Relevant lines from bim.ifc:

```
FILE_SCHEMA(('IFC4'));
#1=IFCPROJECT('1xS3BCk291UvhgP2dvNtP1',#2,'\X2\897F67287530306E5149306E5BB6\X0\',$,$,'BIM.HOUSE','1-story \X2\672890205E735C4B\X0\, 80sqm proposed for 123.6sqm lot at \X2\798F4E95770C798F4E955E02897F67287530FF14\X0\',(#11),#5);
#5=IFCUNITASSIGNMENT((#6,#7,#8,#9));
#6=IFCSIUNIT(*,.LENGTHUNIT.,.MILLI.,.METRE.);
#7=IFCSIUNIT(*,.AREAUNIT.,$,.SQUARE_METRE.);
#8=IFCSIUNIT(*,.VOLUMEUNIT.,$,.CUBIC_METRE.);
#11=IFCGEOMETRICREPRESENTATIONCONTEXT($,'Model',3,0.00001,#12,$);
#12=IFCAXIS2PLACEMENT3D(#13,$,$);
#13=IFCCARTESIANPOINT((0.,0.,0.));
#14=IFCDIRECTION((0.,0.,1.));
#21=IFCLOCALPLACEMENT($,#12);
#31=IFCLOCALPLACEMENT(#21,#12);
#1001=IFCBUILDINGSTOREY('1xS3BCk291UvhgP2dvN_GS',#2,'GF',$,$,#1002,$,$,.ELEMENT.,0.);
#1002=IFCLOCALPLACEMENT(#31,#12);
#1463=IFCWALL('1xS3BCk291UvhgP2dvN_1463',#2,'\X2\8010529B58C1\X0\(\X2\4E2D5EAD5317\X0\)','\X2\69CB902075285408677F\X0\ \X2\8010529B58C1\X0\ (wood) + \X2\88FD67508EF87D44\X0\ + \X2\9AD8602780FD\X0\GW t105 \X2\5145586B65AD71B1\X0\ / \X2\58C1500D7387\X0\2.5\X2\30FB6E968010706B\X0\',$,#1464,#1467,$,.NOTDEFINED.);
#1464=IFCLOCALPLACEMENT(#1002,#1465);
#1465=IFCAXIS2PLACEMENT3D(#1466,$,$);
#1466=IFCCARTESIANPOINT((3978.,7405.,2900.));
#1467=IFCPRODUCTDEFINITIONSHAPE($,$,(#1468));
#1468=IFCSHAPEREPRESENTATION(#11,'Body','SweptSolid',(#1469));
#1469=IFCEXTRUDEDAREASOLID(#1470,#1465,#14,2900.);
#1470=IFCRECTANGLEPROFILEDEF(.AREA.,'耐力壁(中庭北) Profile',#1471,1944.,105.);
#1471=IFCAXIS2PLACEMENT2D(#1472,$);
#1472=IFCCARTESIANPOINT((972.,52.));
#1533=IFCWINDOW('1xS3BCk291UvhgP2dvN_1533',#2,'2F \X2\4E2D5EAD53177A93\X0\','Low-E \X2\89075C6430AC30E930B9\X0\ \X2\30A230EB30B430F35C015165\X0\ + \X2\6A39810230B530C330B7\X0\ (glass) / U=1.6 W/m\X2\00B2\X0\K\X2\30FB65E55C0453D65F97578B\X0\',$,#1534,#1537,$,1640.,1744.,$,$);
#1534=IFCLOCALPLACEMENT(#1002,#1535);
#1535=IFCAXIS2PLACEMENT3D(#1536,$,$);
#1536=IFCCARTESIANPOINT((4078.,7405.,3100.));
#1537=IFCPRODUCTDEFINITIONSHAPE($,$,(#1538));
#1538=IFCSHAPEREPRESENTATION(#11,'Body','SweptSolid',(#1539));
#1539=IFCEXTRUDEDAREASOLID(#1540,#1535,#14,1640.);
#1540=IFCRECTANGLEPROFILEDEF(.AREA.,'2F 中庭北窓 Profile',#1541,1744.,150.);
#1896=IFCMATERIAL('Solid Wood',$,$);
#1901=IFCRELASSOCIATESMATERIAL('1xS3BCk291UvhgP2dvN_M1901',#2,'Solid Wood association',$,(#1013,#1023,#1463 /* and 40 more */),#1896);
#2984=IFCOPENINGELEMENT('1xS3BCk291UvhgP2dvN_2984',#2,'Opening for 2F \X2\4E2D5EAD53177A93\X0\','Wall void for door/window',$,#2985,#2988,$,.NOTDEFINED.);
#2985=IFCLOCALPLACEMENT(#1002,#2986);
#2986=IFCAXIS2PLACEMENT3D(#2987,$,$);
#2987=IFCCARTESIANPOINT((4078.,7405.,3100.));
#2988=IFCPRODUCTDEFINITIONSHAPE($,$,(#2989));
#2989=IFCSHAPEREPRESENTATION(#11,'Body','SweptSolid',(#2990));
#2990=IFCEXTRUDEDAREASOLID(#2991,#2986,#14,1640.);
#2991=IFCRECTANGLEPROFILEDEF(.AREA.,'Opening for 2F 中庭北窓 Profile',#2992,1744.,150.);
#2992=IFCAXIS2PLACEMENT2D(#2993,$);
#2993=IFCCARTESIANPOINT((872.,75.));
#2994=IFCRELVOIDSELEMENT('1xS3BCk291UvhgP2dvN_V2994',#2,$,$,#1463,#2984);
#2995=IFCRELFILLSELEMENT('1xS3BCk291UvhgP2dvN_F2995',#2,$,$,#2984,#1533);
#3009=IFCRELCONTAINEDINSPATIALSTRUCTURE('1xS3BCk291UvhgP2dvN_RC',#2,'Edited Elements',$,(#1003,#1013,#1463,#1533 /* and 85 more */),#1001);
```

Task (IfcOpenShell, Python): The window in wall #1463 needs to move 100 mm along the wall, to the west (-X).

```python
import ifcopenshell
import ifcopenshell.api.geometry
import ifcopenshell.util.placement

model = ifcopenshell.open("bim.ifc")

window = model.by_guid("1xS3BCk291UvhgP2dvN_1533")
opening = window.FillsVoids[0].RelatingOpeningElement
wall = opening.VoidsElements[0].RelatingBuildingElement

wall_matrix = ifcopenshell.util.placement.get_local_placement(wall.ObjectPlacement)
shift = wall_matrix[:3, 0] * -100.0
before = ifcopenshell.util.placement.get_local_placement(window.ObjectPlacement)[:3, 3].copy()

# The window is not placed relative to its opening, so move both.
for product in (opening, window):
    matrix = ifcopenshell.util.placement.get_local_placement(product.ObjectPlacement)
    matrix[:3, 3] += shift
    ifcopenshell.api.geometry.edit_object_placement(model, product=product, matrix=matrix, is_si=False)

after = ifcopenshell.util.placement.get_local_placement(window.ObjectPlacement)[:3, 3]
print("window moved by", (after - before).round(3) + 0.0)

model.write("bim_updated.ifc")
```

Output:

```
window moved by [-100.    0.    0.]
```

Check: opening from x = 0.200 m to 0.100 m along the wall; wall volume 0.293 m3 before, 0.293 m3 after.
